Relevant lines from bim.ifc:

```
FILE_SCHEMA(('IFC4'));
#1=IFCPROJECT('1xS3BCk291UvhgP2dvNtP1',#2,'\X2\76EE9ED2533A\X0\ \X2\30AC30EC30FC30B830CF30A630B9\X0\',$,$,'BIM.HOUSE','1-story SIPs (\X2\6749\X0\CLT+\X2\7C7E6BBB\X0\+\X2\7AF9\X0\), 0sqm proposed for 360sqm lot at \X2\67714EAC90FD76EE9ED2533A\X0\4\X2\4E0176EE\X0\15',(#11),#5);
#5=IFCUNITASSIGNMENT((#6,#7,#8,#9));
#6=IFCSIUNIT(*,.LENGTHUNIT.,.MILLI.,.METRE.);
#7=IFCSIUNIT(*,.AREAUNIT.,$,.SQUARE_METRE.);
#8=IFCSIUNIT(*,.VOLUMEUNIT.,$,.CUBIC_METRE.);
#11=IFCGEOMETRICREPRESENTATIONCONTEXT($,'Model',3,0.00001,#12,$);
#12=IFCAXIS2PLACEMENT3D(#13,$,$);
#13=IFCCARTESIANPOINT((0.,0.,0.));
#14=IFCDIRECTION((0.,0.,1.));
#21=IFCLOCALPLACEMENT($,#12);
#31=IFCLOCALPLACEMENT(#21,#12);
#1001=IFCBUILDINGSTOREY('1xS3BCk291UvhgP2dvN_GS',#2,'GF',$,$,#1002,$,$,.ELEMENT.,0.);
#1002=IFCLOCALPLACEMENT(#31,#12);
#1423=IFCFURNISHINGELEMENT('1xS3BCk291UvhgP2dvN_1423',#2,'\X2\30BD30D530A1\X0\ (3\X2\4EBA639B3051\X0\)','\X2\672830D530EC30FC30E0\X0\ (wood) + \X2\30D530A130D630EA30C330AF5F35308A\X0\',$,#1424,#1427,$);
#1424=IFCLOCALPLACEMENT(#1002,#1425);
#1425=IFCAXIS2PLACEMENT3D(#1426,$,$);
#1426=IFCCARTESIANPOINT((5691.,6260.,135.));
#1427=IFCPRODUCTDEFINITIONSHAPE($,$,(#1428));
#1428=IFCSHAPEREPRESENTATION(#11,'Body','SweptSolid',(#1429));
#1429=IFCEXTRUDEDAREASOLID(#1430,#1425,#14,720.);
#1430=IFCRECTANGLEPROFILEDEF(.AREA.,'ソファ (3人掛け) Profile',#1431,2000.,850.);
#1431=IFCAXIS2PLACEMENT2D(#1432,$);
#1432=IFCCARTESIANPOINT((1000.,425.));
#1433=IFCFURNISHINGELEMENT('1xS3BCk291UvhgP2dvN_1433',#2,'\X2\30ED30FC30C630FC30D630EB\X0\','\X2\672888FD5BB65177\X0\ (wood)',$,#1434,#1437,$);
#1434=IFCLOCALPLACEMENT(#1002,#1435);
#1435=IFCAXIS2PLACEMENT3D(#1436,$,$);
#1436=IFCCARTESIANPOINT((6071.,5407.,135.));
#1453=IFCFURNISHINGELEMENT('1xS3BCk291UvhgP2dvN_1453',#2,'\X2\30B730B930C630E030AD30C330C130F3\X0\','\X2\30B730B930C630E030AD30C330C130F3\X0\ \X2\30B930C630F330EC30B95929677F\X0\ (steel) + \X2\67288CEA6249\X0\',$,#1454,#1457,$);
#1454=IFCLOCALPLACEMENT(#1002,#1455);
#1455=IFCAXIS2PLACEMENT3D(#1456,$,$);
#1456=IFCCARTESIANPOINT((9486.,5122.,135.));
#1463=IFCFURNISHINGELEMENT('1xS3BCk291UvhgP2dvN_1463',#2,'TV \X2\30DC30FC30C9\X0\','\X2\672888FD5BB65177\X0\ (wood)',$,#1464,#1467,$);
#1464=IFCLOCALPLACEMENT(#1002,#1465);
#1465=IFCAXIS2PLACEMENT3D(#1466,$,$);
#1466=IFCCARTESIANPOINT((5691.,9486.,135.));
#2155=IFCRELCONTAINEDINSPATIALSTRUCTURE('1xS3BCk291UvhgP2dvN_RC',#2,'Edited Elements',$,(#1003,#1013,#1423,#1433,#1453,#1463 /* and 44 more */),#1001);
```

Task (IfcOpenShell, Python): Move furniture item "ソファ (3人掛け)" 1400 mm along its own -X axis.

```python
import ifcopenshell
import ifcopenshell.api.geometry
import ifcopenshell.util.placement
import ifcopenshell.util.unit

model = ifcopenshell.open("bim.ifc")
unit_scale = ifcopenshell.util.unit.calculate_unit_scale(model)

item = model.by_guid("1xS3BCk291UvhgP2dvN_1423")
matrix = ifcopenshell.util.placement.get_local_placement(item.ObjectPlacement)
matrix[:3, 3] -= matrix[:3, 0] * 1.4 / unit_scale
ifcopenshell.api.geometry.edit_object_placement(model, product=item, matrix=matrix, is_si=False)

print(ifcopenshell.util.placement.get_local_placement(item.ObjectPlacement).round(3) + 0.0)

model.write("bim-out.ifc")
```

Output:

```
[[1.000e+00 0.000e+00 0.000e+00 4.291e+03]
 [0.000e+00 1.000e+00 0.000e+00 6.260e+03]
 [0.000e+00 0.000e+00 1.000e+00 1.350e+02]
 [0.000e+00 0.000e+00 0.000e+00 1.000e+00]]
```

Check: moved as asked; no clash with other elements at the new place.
